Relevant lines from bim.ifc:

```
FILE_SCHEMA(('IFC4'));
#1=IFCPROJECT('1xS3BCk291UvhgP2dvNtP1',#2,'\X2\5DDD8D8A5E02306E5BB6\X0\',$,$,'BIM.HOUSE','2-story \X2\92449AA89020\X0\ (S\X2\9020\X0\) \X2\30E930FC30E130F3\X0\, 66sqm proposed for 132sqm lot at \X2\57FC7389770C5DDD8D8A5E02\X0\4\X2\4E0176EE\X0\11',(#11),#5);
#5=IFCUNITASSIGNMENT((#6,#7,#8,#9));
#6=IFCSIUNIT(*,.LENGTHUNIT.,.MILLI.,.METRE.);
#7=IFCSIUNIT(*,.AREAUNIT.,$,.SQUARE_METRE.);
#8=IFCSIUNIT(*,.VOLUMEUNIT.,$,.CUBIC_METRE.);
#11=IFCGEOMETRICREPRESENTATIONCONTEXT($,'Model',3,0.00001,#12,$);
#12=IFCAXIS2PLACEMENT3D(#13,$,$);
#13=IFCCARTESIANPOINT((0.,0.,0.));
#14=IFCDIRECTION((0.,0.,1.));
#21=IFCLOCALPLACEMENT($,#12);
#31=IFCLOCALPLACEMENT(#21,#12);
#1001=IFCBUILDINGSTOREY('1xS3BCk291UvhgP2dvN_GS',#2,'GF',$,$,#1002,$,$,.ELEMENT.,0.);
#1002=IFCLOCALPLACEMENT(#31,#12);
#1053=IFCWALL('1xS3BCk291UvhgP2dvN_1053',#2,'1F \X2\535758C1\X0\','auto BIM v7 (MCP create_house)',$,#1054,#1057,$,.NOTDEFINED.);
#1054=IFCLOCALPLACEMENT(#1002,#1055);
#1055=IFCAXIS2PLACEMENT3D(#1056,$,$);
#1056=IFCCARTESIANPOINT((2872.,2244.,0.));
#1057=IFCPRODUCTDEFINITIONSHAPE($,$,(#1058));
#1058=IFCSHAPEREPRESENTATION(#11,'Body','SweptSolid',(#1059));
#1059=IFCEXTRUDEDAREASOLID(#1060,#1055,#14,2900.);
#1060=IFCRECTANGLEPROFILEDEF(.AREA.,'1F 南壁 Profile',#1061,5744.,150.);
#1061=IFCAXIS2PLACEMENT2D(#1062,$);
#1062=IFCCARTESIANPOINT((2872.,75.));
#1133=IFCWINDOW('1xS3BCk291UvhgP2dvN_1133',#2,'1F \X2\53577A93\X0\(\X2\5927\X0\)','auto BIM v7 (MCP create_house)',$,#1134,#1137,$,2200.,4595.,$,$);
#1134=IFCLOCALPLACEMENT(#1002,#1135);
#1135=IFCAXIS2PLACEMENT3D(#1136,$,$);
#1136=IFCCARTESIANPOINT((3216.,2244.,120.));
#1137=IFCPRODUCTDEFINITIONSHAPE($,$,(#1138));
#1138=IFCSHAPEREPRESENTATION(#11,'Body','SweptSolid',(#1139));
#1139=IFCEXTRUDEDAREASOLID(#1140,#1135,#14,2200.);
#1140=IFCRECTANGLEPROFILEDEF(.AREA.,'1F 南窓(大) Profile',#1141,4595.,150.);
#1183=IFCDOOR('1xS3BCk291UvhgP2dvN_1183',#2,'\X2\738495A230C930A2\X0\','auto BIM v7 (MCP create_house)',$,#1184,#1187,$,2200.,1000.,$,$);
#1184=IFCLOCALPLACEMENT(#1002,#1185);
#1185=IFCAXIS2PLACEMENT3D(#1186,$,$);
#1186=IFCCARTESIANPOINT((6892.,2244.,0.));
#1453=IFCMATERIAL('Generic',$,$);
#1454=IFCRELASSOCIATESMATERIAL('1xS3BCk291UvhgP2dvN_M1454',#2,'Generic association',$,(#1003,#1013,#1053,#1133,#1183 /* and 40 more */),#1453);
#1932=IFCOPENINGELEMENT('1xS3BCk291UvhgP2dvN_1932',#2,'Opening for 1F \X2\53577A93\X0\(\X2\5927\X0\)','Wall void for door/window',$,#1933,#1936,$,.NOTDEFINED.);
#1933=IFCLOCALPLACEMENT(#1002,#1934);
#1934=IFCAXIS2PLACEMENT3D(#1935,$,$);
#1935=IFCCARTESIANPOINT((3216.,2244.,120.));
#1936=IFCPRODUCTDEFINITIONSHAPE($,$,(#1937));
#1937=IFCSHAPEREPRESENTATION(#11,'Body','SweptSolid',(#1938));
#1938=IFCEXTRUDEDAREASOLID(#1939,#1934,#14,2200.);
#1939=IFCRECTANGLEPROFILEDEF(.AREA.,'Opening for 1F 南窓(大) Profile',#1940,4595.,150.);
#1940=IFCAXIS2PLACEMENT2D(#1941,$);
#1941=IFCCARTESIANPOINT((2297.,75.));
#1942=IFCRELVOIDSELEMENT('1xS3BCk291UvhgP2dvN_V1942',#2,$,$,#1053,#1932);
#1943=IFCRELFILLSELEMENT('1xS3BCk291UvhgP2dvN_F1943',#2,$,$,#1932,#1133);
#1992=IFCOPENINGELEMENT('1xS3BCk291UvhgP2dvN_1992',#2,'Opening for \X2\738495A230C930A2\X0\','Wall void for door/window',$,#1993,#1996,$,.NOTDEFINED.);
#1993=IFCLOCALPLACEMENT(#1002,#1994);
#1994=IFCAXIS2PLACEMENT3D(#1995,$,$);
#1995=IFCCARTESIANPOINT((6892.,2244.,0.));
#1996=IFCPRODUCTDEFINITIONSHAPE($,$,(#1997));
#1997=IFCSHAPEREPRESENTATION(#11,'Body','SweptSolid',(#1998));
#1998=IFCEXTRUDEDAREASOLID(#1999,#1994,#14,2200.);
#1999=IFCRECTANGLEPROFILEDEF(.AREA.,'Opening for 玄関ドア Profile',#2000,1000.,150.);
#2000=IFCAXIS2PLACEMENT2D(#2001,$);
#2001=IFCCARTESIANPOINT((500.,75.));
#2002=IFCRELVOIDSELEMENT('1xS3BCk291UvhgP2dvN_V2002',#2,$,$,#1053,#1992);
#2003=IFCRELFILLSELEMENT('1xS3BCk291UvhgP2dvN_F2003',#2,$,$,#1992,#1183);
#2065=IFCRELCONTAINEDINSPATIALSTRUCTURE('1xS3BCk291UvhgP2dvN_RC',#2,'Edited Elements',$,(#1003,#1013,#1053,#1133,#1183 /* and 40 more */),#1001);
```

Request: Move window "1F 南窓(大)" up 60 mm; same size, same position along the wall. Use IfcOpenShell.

```python
import numpy as np
import ifcopenshell
import ifcopenshell.api.geometry
import ifcopenshell.util.placement
import ifcopenshell.util.unit

model = ifcopenshell.open("bim.ifc")
unit_scale = ifcopenshell.util.unit.calculate_unit_scale(model)

window = model.by_guid("1xS3BCk291UvhgP2dvN_1133")
opening = window.FillsVoids[0].RelatingOpeningElement
dz = 0.06 / unit_scale

shift = np.array([0.0, 0.0, dz])
# The window is not placed relative to its opening, so move both.
for product in (opening, window):
    matrix = ifcopenshell.util.placement.get_local_placement(product.ObjectPlacement)
    matrix[:3, 3] += shift
    ifcopenshell.api.geometry.edit_object_placement(model, product=product, matrix=matrix, is_si=False)

print(f"moved by {dz * unit_scale:+.3f} m")

model.write("bim_updated.ifc")
```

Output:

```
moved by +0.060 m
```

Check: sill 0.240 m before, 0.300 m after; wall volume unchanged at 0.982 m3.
